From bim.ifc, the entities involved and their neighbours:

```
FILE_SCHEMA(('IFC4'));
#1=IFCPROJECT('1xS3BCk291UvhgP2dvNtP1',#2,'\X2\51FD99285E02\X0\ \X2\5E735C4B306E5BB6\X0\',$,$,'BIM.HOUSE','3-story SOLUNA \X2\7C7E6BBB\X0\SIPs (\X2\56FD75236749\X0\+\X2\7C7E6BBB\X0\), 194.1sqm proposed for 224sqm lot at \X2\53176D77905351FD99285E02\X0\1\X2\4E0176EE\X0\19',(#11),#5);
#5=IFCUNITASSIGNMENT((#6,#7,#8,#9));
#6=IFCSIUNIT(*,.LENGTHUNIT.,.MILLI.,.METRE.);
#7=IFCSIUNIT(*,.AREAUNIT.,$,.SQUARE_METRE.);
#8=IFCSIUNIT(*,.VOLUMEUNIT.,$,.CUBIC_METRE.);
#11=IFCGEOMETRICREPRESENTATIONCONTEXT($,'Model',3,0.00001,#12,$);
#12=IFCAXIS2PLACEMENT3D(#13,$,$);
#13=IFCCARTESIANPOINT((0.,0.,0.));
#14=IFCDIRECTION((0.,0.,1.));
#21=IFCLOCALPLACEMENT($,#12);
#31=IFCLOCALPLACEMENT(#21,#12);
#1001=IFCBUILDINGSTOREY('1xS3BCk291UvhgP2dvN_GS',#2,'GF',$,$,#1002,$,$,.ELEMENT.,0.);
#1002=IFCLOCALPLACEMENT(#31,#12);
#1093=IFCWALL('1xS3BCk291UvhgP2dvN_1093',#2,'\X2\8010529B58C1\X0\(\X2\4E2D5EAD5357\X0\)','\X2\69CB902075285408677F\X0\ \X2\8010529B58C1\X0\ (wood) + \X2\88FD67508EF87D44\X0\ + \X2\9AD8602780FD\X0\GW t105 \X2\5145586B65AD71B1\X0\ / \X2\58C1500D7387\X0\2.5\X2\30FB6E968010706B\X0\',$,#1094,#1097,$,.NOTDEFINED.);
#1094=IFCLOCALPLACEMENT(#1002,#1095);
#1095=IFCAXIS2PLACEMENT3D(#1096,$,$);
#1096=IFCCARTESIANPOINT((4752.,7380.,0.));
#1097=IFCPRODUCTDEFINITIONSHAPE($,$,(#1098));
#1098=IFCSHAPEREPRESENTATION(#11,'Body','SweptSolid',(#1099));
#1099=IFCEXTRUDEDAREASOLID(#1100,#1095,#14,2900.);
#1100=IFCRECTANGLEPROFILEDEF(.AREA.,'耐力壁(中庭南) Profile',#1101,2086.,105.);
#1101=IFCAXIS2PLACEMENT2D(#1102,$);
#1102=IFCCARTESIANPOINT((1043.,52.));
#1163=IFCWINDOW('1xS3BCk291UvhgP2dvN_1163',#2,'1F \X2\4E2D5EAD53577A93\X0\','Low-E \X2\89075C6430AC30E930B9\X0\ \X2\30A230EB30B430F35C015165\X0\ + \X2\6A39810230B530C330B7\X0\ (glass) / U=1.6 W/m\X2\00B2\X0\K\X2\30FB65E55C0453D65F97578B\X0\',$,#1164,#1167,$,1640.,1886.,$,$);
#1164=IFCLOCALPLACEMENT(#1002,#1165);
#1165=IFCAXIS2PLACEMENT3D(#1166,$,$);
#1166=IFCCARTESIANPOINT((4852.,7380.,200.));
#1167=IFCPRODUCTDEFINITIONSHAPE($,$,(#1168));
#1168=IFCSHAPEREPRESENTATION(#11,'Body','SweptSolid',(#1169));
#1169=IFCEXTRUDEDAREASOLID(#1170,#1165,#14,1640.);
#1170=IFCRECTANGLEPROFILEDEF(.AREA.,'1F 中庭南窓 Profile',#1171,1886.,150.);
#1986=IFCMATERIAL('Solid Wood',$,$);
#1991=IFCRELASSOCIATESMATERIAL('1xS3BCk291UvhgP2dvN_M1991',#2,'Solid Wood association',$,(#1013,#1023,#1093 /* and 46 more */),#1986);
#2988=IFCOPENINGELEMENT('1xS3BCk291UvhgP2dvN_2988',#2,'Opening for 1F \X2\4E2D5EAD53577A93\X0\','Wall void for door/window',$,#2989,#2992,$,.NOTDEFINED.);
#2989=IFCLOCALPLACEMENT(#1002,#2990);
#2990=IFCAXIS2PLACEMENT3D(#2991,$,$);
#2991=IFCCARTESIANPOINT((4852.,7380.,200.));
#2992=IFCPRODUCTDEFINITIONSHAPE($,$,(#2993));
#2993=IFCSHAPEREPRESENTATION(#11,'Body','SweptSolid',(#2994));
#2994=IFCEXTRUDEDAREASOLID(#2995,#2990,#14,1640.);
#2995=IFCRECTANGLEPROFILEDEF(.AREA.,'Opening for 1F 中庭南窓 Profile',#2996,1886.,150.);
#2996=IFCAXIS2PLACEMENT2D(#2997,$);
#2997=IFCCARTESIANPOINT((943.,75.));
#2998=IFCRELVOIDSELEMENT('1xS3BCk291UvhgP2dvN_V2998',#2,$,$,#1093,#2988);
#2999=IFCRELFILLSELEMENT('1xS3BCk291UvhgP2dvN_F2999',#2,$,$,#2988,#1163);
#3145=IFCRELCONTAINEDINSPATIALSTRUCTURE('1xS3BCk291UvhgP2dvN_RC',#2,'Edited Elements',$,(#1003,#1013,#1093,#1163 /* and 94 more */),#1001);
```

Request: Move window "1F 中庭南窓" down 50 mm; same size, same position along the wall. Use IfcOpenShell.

```python
import numpy as np
import ifcopenshell
import ifcopenshell.api.geometry
import ifcopenshell.util.placement
import ifcopenshell.util.unit

model = ifcopenshell.open("bim.ifc")
unit_scale = ifcopenshell.util.unit.calculate_unit_scale(model)

window = model.by_guid("1xS3BCk291UvhgP2dvN_1163")
opening = window.FillsVoids[0].RelatingOpeningElement
dz = -0.05 / unit_scale

shift = np.array([0.0, 0.0, dz])
# The window is not placed relative to its opening, so move both.
for product in (opening, window):
    matrix = ifcopenshell.util.placement.get_local_placement(product.ObjectPlacement)
    matrix[:3, 3] += shift
    ifcopenshell.api.geometry.edit_object_placement(model, product=product, matrix=matrix, is_si=False)

print(f"moved by {dz * unit_scale:+.3f} m")

model.write("bim_edited.ifc")
```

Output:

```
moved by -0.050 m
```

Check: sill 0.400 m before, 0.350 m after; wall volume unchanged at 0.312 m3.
